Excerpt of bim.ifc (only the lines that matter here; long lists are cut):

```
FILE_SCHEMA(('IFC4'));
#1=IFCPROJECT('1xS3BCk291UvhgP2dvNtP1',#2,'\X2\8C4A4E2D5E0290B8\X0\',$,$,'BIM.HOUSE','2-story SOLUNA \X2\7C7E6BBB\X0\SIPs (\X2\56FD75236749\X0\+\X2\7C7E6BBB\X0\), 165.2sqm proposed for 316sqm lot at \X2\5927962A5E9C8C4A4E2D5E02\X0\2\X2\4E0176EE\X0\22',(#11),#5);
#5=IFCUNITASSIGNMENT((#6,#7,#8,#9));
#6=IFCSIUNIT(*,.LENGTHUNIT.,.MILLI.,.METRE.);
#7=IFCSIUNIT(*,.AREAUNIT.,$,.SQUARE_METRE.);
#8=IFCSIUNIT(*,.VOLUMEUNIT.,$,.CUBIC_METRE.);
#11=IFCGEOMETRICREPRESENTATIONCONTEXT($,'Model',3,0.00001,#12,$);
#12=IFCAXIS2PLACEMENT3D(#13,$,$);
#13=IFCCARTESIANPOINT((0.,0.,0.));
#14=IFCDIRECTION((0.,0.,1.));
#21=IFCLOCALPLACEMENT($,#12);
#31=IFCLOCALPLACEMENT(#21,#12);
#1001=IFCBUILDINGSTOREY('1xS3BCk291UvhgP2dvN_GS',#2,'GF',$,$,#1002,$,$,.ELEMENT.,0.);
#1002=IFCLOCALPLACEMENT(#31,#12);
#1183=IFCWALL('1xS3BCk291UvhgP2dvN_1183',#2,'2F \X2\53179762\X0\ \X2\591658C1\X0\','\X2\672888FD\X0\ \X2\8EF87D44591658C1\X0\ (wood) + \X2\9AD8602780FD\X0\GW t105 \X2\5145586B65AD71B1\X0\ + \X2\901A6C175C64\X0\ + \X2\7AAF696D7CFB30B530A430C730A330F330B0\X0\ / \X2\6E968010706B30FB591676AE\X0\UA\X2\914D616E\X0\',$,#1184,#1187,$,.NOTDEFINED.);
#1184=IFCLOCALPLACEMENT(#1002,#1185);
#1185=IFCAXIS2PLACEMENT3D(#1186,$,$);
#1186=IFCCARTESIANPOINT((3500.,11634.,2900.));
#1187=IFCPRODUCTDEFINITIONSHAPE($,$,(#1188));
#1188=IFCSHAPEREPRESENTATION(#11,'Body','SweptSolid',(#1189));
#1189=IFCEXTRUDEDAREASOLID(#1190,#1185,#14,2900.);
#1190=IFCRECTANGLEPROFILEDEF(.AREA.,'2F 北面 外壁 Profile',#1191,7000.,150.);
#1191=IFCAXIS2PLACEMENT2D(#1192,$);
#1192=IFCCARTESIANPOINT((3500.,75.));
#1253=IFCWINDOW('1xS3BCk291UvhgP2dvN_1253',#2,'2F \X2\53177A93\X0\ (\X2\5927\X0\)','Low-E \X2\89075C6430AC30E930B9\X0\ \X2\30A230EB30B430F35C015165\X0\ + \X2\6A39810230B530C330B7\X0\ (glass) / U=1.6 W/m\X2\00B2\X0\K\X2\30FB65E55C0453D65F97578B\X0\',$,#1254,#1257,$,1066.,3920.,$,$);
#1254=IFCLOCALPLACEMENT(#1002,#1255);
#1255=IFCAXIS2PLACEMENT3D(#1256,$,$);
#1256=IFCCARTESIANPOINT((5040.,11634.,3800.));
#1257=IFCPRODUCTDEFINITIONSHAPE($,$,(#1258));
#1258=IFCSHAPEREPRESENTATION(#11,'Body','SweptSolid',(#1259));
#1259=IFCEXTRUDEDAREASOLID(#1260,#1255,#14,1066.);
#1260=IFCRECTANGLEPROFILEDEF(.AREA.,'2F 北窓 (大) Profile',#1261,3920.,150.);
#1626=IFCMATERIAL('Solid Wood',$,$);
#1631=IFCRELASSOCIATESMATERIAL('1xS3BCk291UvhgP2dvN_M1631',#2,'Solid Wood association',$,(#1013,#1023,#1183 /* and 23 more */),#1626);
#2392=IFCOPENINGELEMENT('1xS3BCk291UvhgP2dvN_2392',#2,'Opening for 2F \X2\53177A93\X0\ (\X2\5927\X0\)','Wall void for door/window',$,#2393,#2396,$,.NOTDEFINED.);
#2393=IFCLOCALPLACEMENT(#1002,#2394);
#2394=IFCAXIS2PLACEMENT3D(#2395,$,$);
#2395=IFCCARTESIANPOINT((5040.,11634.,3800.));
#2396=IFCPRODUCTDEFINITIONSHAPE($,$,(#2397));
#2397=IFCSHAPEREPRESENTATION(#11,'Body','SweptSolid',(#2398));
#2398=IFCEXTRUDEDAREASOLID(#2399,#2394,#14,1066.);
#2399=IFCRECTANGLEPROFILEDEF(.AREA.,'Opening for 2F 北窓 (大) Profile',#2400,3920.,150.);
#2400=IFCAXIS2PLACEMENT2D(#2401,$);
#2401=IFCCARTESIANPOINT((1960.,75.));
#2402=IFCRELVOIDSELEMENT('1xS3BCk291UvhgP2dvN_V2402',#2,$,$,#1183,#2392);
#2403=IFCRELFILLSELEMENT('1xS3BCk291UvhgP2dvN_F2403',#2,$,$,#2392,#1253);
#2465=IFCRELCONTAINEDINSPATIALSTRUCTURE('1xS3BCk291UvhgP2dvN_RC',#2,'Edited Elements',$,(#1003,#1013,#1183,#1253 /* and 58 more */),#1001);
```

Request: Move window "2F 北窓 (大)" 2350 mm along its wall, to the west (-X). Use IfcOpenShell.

```python
import ifcopenshell
import ifcopenshell.api.geometry
import ifcopenshell.util.placement

model = ifcopenshell.open("bim.ifc")

window = model.by_id(1253)
opening = window.FillsVoids[0].RelatingOpeningElement
wall = opening.VoidsElements[0].RelatingBuildingElement

wall_matrix = ifcopenshell.util.placement.get_local_placement(wall.ObjectPlacement)
shift = wall_matrix[:3, 0] * -2350.0
before = ifcopenshell.util.placement.get_local_placement(window.ObjectPlacement)[:3, 3].copy()

# The window is not placed relative to its opening, so move both.
for product in (opening, window):
    matrix = ifcopenshell.util.placement.get_local_placement(product.ObjectPlacement)
    matrix[:3, 3] += shift
    ifcopenshell.api.geometry.edit_object_placement(model, product=product, matrix=matrix, is_si=False)

after = ifcopenshell.util.placement.get_local_placement(window.ObjectPlacement)[:3, 3]
print("window moved by", (after - before).round(3) + 0.0)

model.write("bim-out.ifc")
```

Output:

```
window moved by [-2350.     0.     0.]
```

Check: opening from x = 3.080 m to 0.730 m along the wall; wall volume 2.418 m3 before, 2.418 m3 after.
